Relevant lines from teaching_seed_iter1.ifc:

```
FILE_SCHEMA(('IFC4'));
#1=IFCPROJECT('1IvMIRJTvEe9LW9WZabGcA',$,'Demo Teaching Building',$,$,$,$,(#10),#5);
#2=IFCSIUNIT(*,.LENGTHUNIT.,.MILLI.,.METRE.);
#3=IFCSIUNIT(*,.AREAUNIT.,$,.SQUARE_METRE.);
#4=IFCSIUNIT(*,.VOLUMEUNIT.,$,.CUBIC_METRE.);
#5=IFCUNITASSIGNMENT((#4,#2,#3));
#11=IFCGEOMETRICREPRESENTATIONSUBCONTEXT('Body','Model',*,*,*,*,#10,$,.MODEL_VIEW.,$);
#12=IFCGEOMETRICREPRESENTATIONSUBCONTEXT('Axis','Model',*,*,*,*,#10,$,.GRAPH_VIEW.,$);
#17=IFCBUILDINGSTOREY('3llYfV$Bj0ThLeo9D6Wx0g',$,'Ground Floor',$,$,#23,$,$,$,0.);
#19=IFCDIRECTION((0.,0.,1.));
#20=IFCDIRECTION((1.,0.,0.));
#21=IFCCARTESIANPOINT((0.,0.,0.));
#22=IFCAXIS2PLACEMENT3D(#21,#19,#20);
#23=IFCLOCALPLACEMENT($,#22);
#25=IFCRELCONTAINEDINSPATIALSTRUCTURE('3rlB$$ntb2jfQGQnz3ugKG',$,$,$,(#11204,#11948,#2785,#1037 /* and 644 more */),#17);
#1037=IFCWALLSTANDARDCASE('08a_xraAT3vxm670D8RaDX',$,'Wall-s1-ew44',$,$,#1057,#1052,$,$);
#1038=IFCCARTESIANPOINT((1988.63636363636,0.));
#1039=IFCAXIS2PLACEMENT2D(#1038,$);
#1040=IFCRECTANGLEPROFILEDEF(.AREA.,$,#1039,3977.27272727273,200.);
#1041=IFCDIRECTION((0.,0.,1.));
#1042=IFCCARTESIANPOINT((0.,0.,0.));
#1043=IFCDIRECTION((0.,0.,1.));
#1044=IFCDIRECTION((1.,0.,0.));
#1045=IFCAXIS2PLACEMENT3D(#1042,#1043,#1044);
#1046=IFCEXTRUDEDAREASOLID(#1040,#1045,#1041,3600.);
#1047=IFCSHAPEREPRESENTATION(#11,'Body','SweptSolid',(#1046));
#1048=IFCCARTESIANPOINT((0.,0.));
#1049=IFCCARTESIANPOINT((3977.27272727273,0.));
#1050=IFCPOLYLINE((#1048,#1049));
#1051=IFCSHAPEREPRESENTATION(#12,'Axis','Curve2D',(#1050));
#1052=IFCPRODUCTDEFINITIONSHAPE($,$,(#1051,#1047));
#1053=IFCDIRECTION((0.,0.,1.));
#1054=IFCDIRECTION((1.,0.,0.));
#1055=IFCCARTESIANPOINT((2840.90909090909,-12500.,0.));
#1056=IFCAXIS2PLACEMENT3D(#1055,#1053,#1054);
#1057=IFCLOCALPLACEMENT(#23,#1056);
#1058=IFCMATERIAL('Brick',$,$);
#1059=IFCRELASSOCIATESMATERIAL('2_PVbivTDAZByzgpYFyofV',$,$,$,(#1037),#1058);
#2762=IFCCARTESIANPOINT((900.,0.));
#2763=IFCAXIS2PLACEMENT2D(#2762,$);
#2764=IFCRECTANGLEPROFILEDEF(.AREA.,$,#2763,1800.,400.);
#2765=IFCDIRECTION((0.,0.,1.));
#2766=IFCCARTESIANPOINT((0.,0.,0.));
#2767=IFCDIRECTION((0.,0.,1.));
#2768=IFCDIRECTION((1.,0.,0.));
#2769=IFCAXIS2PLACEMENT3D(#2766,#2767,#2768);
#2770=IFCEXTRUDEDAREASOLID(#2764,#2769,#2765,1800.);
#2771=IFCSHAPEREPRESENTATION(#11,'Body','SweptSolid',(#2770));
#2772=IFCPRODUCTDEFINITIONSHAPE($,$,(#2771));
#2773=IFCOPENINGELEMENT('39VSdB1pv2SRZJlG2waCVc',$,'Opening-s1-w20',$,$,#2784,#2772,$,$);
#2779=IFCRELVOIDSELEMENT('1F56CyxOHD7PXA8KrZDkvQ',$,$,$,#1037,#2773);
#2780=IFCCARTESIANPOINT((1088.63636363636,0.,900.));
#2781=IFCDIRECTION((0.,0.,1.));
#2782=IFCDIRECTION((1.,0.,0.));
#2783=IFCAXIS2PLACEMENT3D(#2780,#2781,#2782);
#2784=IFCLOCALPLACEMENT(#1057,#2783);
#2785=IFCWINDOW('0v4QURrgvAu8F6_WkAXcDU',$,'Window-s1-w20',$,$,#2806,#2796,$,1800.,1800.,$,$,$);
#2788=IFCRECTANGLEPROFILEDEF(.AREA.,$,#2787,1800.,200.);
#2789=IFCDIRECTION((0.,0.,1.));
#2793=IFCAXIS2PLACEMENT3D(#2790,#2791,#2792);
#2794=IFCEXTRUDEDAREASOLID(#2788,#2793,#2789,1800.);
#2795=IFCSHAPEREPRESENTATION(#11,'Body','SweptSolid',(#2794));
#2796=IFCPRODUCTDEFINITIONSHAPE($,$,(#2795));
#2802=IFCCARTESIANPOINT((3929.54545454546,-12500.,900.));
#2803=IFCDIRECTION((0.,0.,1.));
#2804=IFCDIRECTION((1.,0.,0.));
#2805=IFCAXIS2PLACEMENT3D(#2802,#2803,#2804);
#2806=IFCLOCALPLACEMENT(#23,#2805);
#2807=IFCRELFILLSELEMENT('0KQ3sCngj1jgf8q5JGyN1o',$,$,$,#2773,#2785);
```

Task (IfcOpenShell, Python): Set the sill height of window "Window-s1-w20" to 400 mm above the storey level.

```python
import numpy as np
import ifcopenshell
import ifcopenshell.api.geometry
import ifcopenshell.geom
import ifcopenshell.util.element
import ifcopenshell.util.placement
import ifcopenshell.util.shape
import ifcopenshell.util.unit

model = ifcopenshell.open("teaching_seed_iter1.ifc")
unit_scale = ifcopenshell.util.unit.calculate_unit_scale(model)

window = model.by_guid("0v4QURrgvAu8F6_WkAXcDU")
opening = window.FillsVoids[0].RelatingOpeningElement
storey = ifcopenshell.util.element.get_container(window, ifc_class="IfcBuildingStorey")
level = ifcopenshell.util.placement.get_local_placement(storey.ObjectPlacement)[2, 3]

# The opening's origin need not be at the sill, so measure its lowest point.
shape = ifcopenshell.geom.create_shape(ifcopenshell.geom.settings(), opening)
bottom = ifcopenshell.util.shape.get_shape_bottom_elevation(shape, shape.geometry) / unit_scale
dz = level + 400.0 - bottom

shift = np.array([0.0, 0.0, dz])
# The window is not placed relative to its opening, so move both.
for product in (opening, window):
    matrix = ifcopenshell.util.placement.get_local_placement(product.ObjectPlacement)
    matrix[:3, 3] += shift
    ifcopenshell.api.geometry.edit_object_placement(model, product=product, matrix=matrix, is_si=False)

print(f"moved by {dz * unit_scale:+.3f} m")

model.write("teaching_seed_iter1_rev.ifc")
```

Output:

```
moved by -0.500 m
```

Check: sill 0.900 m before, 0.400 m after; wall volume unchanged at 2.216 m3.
